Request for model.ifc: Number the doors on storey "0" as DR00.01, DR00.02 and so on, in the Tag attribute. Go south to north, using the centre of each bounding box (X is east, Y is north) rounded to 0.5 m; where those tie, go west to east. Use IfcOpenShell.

First a look at what the model holds.

```python
import ifcopenshell
import ifcopenshell.util.element
import ifcopenshell.util.placement

model = ifcopenshell.open("model.ifc")
print(model.schema)
storey = next(s for s in model.by_type("IfcBuildingStorey") if s.Name == "0")
doors = [e for e in ifcopenshell.util.element.get_decomposition(storey) if e.is_a("IfcDoor")]
for e in sorted(doors, key=lambda e: e.id()):
    origin = ifcopenshell.util.placement.get_local_placement(e.ObjectPlacement)[:3, 3]
    print(e.id(), e.Tag, e.Name, origin.round(2) + 0.0, sep=" | ")
```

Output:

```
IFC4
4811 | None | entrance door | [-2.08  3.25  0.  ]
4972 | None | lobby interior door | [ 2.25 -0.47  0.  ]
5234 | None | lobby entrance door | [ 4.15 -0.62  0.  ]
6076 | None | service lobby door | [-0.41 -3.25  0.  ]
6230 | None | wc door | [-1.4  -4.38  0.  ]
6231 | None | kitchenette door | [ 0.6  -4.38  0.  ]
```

```python
import ifcopenshell
import ifcopenshell.geom
import ifcopenshell.util.element
import ifcopenshell.util.shape

model = ifcopenshell.open("model.ifc")
settings = ifcopenshell.geom.settings()
settings.set("use-world-coords", True)


def centre(element):
    shape = ifcopenshell.geom.create_shape(settings, element)
    return ifcopenshell.util.shape.get_bbox_centroid(shape.geometry)


storey = next(s for s in model.by_type("IfcBuildingStorey") if s.Name == "0")
doors = [e for e in ifcopenshell.util.element.get_decomposition(storey) if e.is_a("IfcDoor")]

# Insertion points can sit at a corner or the storey origin, so sort by the geometry (in metres).
centres = {e: centre(e) for e in doors}
doors.sort(key=lambda e: (round(centres[e][1] / 0.5), centres[e][0]))

for i, e in enumerate(doors, start=1):
    number = f"DR00.{i:02d}"
    e.Tag = number
    print(e.id(), number)

model.write("model-out.ifc")
```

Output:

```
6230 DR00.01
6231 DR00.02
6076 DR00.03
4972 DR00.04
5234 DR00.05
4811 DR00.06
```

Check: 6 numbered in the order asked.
